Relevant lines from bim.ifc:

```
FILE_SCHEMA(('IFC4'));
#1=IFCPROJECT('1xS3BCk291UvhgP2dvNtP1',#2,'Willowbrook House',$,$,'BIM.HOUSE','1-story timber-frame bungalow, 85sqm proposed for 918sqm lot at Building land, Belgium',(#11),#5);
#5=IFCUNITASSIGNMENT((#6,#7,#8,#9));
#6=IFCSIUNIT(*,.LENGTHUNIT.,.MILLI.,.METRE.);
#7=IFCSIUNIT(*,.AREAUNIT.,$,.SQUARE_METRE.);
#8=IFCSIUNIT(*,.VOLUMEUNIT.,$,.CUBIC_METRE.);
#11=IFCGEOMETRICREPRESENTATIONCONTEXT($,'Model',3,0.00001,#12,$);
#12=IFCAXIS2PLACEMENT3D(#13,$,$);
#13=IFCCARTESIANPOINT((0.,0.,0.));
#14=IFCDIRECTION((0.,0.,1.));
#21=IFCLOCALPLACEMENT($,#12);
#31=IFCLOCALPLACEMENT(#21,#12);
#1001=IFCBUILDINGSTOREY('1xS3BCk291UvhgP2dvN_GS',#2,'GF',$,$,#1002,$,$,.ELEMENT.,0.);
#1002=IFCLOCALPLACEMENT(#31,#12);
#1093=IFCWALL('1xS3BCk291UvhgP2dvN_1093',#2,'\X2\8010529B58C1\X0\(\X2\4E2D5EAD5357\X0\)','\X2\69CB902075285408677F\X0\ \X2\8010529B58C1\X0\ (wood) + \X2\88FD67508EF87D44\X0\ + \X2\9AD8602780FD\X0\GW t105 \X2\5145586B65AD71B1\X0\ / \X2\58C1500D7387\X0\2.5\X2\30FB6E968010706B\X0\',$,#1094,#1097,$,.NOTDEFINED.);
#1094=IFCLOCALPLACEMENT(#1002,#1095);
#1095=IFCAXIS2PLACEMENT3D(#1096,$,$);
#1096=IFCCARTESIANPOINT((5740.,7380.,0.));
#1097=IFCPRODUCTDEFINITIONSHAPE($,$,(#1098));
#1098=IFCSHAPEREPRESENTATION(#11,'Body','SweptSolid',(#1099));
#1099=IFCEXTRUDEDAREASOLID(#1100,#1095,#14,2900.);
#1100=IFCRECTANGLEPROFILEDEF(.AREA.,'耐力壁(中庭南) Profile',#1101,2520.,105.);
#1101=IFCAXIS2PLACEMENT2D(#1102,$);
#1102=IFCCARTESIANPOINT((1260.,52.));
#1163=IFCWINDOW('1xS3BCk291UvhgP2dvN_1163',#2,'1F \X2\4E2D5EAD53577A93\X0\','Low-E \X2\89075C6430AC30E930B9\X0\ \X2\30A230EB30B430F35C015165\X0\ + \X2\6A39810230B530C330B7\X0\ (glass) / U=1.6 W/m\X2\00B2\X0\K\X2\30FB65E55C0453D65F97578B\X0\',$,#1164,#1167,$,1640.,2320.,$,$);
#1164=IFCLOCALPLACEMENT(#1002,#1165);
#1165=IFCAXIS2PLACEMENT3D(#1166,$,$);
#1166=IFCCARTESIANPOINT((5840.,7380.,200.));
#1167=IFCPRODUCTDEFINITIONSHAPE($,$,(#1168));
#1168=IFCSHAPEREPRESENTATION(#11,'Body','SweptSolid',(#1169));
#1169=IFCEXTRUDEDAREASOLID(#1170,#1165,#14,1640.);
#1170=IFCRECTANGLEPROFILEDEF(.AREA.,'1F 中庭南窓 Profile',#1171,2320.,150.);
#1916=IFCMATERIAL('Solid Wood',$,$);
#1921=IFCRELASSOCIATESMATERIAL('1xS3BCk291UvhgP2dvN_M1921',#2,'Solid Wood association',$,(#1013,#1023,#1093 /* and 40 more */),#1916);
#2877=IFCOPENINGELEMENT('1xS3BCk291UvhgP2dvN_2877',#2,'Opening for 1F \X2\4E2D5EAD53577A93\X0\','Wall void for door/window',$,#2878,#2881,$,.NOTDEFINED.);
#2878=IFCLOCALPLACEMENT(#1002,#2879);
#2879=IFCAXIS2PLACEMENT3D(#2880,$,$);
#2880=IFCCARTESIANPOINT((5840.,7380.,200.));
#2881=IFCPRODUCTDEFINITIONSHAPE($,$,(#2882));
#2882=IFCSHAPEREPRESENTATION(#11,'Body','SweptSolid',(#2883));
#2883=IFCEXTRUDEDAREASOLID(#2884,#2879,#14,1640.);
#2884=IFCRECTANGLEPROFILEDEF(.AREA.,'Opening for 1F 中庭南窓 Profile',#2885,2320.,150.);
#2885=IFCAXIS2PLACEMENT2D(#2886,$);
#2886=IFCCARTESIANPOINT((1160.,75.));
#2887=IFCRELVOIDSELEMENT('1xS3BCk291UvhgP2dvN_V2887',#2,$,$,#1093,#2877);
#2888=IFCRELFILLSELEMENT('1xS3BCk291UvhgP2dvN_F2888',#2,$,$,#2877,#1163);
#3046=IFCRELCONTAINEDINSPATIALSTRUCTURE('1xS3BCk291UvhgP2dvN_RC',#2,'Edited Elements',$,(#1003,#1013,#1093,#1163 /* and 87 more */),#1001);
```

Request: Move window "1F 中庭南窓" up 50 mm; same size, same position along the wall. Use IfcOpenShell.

```python
import numpy as np
import ifcopenshell
import ifcopenshell.api.geometry
import ifcopenshell.util.placement
import ifcopenshell.util.unit

model = ifcopenshell.open("bim.ifc")
unit_scale = ifcopenshell.util.unit.calculate_unit_scale(model)

window = model.by_guid("1xS3BCk291UvhgP2dvN_1163")
opening = window.FillsVoids[0].RelatingOpeningElement
dz = 0.05 / unit_scale

shift = np.array([0.0, 0.0, dz])
# The window is not placed relative to its opening, so move both.
for product in (opening, window):
    matrix = ifcopenshell.util.placement.get_local_placement(product.ObjectPlacement)
    matrix[:3, 3] += shift
    ifcopenshell.api.geometry.edit_object_placement(model, product=product, matrix=matrix, is_si=False)

print(f"moved by {dz * unit_scale:+.3f} m")

model.write("bim-out.ifc")
```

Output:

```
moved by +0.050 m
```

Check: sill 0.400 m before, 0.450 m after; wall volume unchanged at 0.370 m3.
